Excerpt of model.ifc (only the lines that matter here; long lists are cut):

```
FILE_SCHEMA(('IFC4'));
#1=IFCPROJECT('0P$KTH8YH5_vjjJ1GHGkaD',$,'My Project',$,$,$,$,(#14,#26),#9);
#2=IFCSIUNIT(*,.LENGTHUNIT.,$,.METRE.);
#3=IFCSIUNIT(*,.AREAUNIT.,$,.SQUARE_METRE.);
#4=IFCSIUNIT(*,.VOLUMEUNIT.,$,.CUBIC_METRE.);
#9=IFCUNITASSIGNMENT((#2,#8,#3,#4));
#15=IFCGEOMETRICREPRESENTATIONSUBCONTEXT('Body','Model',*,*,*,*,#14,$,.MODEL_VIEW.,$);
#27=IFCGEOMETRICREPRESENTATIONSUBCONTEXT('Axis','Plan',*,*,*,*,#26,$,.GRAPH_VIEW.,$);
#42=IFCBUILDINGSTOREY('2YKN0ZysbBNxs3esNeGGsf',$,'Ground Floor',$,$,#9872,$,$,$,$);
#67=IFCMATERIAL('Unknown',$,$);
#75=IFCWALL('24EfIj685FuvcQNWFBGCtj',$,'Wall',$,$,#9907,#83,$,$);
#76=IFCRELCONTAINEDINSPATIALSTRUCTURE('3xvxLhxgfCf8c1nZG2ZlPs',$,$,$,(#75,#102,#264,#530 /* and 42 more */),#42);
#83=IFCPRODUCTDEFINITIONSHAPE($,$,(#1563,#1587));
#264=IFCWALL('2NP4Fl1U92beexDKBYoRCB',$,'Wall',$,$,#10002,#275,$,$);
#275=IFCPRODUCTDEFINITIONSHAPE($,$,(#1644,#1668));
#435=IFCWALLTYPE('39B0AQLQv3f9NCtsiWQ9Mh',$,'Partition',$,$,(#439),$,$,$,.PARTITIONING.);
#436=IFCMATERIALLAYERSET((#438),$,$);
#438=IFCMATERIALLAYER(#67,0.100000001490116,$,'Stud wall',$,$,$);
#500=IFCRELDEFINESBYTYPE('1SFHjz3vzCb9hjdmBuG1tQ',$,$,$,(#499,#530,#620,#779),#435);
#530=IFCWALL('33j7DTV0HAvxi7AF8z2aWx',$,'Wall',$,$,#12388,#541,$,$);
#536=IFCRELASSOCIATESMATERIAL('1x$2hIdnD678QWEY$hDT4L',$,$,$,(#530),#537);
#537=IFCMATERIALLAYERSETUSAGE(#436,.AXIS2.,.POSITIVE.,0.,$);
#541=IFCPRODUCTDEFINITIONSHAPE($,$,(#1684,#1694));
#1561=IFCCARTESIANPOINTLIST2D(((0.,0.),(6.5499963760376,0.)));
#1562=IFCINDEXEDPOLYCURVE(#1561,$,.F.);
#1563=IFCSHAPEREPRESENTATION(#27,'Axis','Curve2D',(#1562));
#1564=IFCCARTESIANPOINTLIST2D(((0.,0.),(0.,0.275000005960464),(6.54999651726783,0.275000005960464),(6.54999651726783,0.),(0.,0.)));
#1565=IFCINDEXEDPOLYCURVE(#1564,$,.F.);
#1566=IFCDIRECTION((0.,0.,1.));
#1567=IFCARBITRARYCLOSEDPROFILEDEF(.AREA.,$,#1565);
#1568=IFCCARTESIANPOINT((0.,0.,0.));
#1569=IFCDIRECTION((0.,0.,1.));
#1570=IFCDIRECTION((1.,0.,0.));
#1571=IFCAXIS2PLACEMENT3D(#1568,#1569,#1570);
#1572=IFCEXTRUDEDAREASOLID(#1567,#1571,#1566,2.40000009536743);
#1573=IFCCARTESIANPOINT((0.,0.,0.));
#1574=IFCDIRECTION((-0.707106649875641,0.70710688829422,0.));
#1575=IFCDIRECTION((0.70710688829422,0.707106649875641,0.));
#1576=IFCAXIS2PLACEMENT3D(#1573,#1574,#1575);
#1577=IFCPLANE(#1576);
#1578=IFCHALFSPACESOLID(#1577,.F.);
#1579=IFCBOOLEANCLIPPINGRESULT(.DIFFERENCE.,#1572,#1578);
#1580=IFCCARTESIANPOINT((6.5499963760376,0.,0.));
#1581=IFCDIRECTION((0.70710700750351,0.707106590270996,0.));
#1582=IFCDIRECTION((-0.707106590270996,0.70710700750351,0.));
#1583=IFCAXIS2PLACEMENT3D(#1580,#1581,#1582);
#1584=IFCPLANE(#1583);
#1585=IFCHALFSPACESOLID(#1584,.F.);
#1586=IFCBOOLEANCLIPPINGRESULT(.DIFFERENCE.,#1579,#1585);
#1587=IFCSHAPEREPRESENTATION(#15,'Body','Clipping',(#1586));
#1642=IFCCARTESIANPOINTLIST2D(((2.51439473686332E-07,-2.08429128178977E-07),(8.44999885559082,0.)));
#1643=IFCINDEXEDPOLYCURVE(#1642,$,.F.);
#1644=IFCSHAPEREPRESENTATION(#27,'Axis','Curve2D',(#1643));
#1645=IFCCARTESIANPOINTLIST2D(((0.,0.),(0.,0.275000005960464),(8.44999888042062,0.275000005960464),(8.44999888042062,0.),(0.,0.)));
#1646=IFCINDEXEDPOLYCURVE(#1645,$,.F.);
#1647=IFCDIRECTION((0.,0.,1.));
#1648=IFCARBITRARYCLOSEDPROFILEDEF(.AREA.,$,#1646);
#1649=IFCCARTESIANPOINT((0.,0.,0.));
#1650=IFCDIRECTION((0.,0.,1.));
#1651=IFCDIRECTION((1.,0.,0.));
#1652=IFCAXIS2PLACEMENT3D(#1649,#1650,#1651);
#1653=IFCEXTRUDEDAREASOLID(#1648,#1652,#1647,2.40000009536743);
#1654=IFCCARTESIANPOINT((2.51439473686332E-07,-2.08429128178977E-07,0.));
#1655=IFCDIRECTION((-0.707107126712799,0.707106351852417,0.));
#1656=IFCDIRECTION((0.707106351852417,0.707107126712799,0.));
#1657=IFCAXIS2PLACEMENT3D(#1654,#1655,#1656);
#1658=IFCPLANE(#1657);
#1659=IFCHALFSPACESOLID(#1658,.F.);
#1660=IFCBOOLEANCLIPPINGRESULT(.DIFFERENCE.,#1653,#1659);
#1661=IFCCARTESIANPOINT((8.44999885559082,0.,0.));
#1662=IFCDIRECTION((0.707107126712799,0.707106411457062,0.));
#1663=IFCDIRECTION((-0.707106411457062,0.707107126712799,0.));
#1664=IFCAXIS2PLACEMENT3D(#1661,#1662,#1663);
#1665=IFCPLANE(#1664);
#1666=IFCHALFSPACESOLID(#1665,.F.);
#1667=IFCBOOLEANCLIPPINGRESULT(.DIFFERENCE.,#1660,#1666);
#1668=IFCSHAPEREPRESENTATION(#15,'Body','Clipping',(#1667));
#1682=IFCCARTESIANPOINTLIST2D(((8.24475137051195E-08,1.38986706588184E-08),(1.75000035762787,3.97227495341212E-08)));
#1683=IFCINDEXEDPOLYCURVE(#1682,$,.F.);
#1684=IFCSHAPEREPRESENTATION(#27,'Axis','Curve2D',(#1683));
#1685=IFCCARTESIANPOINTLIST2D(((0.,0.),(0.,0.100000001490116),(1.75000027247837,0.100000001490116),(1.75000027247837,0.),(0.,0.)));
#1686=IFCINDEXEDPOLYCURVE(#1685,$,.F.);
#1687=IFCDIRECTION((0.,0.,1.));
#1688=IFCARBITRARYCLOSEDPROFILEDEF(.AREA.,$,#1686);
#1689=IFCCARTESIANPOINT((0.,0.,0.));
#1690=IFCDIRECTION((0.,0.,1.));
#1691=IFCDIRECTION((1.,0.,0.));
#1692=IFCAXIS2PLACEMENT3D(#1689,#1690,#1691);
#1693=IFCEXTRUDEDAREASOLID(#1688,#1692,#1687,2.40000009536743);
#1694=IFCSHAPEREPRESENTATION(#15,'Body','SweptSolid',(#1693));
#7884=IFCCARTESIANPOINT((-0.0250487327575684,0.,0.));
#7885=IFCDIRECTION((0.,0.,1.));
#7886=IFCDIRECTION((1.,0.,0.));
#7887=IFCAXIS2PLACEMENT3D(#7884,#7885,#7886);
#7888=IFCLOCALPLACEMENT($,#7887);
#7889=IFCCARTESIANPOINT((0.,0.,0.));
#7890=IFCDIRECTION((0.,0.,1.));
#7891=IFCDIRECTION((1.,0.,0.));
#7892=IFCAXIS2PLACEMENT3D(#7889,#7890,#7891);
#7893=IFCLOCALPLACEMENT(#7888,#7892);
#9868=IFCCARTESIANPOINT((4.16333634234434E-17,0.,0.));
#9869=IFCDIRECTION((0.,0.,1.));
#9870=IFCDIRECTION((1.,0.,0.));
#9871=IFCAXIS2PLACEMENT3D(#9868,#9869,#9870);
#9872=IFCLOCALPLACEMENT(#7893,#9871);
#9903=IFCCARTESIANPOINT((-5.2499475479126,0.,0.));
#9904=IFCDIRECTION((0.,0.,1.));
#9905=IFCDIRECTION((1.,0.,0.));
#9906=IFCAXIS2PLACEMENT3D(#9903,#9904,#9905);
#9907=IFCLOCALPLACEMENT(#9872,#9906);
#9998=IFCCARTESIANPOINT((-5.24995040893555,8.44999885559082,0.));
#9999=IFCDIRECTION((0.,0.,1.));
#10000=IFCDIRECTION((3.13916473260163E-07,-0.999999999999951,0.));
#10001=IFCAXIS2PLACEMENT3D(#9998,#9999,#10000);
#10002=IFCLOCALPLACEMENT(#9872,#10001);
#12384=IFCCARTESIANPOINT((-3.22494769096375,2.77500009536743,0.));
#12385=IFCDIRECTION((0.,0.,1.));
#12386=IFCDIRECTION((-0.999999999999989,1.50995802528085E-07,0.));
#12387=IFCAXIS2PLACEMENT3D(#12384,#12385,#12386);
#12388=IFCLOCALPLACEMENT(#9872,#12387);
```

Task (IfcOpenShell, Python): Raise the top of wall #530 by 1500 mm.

```python
import ifcopenshell
import ifcopenshell.geom
import ifcopenshell.util.representation
import ifcopenshell.util.shape

model = ifcopenshell.open("model.ifc")
settings = ifcopenshell.geom.settings()


def volume(element):
    """Net volume in cubic metres, openings subtracted."""
    shape = ifcopenshell.geom.create_shape(settings, element)
    return ifcopenshell.util.shape.get_volume(shape.geometry)


wall = model.by_id(530)
before = volume(wall)

body = ifcopenshell.util.representation.get_representation(wall, "Model", "Body")
solid = body.Items[0]
old_height = solid.Depth
solid.Depth += 1.5
after = volume(wall)

print(f"height {old_height:g} -> {solid.Depth:g}, volume {before:.3f} -> {after:.3f} m3")

model.write("model-out.ifc")
```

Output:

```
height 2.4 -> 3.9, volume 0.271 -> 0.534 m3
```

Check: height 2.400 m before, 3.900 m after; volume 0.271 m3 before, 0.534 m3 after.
